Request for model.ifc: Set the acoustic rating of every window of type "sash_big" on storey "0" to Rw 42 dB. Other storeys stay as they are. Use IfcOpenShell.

First a look at what the model holds.

```python
import ifcopenshell
import ifcopenshell.util.element

model = ifcopenshell.open("model.ifc")
print(model.schema)
storey = next(s for s in model.by_type("IfcBuildingStorey") if s.Name == "0")
windows = [e for e in ifcopenshell.util.element.get_decomposition(storey) if e.is_a("IfcWindow")]
seen = {}
for e in windows:
    element_type = ifcopenshell.util.element.get_type(e)
    key = (element_type.Name if element_type != e and element_type else None, ifcopenshell.util.element.get_pset(e, "Pset_WindowCommon", "AcousticRating"))
    seen[key] = seen.get(key, 0) + 1
for (name, value), count in sorted(seen.items(), key=str):
    print(count, "x", name, "|", value)
```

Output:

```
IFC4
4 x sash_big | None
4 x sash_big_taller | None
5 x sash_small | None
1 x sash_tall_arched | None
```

```python
import ifcopenshell
import ifcopenshell.api.pset
import ifcopenshell.util.element

model = ifcopenshell.open("model.ifc")

storey = next(s for s in model.by_type("IfcBuildingStorey") if s.Name == "0")
windows = [e for e in ifcopenshell.util.element.get_decomposition(storey) if e.is_a("IfcWindow")]

count = 0
for e in windows:
    element_type = ifcopenshell.util.element.get_type(e)
    if element_type in (None, e) or element_type.Name != "sash_big":
        continue
    # add_pset returns the element's existing set when there is one.
    pset = ifcopenshell.api.pset.add_pset(model, product=e, name="Pset_WindowCommon")
    ifcopenshell.api.pset.edit_pset(model, pset=pset, properties={"AcousticRating": "Rw 42 dB"})
    count += 1

print(count, "windows updated")

model.write("model_updated.ifc")
```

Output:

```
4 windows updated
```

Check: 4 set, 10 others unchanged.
